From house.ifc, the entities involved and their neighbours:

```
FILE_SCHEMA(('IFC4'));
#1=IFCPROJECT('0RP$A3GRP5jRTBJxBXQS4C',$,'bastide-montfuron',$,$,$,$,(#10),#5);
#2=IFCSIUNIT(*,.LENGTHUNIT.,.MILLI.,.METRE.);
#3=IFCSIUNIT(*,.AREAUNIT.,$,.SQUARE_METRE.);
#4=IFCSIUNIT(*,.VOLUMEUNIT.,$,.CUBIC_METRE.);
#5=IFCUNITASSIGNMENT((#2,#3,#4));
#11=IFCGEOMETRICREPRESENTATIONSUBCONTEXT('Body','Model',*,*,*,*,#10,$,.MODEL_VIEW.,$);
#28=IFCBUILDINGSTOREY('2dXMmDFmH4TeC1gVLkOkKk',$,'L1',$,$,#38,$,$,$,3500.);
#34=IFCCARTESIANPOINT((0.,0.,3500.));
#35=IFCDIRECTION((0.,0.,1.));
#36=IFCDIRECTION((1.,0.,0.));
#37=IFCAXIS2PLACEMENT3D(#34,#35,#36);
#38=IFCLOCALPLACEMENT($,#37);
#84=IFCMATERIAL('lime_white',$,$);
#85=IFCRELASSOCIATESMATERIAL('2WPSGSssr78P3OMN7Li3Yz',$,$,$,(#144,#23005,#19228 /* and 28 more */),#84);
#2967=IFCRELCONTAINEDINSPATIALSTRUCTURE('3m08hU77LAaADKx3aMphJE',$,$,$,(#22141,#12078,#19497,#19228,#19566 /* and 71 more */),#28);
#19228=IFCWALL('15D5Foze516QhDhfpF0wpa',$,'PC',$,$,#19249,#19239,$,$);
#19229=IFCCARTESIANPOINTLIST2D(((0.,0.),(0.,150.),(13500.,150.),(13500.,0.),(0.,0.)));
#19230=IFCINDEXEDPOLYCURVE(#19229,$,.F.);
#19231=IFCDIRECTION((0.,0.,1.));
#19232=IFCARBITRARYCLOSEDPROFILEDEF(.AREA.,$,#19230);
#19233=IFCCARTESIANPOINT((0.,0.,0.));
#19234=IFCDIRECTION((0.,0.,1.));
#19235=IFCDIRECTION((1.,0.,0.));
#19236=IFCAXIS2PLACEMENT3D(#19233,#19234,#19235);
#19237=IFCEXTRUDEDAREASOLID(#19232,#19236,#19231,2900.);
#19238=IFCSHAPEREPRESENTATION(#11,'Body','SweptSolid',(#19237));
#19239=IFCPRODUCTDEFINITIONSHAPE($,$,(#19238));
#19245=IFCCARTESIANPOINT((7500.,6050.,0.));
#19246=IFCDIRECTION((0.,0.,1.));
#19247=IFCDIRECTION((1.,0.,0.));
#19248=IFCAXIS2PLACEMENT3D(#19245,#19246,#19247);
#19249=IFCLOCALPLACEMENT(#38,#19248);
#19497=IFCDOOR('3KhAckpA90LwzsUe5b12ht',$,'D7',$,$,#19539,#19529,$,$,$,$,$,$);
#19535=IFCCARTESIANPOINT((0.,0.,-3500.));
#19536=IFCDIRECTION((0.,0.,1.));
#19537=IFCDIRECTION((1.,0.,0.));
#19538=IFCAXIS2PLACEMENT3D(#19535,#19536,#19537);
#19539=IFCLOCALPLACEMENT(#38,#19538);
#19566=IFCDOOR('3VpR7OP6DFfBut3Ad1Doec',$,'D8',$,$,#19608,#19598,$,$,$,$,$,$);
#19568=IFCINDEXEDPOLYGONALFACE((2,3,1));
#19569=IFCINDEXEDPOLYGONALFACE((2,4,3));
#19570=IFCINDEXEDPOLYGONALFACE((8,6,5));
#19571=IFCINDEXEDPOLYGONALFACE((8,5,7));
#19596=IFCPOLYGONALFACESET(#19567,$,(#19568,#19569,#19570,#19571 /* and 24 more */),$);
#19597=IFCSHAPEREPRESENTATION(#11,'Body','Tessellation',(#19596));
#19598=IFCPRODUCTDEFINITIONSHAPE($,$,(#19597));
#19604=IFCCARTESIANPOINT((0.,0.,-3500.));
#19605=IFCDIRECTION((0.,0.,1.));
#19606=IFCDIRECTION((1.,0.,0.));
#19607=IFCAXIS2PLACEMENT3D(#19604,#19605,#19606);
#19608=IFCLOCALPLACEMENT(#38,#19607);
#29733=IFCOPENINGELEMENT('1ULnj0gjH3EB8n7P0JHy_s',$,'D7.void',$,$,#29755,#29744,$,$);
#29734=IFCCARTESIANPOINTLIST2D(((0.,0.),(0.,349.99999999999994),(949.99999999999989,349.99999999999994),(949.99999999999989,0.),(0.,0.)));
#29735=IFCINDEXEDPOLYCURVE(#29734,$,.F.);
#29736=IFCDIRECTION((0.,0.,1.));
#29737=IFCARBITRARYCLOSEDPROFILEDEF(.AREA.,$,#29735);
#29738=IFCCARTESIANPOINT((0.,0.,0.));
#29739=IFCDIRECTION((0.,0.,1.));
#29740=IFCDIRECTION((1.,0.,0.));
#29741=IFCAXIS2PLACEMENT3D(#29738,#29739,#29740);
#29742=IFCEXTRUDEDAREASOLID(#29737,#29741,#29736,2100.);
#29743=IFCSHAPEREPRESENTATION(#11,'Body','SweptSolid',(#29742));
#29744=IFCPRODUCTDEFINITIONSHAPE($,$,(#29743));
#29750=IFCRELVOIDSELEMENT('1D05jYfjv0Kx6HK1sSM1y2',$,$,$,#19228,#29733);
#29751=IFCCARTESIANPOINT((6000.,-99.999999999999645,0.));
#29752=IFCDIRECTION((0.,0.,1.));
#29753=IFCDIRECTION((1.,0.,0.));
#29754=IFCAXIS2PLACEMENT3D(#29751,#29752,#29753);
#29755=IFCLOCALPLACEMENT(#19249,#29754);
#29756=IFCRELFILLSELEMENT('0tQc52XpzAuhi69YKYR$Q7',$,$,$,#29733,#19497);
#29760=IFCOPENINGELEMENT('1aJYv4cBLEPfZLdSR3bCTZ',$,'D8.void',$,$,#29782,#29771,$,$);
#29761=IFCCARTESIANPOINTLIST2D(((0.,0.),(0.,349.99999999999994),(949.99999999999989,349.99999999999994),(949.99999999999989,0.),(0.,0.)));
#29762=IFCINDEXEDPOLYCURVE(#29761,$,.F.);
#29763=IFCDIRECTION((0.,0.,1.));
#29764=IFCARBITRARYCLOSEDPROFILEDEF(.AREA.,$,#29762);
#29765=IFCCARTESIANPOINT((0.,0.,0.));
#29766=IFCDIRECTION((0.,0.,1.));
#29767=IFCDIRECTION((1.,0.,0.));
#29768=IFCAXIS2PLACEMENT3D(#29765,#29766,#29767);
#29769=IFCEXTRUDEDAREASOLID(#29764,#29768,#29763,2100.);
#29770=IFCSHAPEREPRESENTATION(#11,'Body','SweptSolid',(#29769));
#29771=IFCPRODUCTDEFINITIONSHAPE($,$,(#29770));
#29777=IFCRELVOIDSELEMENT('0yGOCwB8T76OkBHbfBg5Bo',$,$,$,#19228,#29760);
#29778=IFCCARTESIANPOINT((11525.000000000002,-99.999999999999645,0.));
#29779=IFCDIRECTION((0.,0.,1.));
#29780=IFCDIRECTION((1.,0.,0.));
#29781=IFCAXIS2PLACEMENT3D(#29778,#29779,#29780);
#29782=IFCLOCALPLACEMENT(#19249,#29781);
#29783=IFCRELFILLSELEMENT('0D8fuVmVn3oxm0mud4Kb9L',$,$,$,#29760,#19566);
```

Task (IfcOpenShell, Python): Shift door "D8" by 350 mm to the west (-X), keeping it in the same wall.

```python
import ifcopenshell
import ifcopenshell.api.geometry
import ifcopenshell.util.placement
import ifcopenshell.util.unit

model = ifcopenshell.open("house.ifc")
unit_scale = ifcopenshell.util.unit.calculate_unit_scale(model)

door = model.by_guid("3VpR7OP6DFfBut3Ad1Doec")
opening = door.FillsVoids[0].RelatingOpeningElement
wall = opening.VoidsElements[0].RelatingBuildingElement

wall_matrix = ifcopenshell.util.placement.get_local_placement(wall.ObjectPlacement)
shift = wall_matrix[:3, 0] * -0.35 / unit_scale
before = ifcopenshell.util.placement.get_local_placement(door.ObjectPlacement)[:3, 3].copy()

# The door is not placed relative to its opening, so move both.
for product in (opening, door):
    matrix = ifcopenshell.util.placement.get_local_placement(product.ObjectPlacement)
    matrix[:3, 3] += shift
    ifcopenshell.api.geometry.edit_object_placement(model, product=product, matrix=matrix, is_si=False)

after = ifcopenshell.util.placement.get_local_placement(door.ObjectPlacement)[:3, 3]
print("door moved by", (after - before).round(3) + 0.0)

model.write("house_edited.ifc")
```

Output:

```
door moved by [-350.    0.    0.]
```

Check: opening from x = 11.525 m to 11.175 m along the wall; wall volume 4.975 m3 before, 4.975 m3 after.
